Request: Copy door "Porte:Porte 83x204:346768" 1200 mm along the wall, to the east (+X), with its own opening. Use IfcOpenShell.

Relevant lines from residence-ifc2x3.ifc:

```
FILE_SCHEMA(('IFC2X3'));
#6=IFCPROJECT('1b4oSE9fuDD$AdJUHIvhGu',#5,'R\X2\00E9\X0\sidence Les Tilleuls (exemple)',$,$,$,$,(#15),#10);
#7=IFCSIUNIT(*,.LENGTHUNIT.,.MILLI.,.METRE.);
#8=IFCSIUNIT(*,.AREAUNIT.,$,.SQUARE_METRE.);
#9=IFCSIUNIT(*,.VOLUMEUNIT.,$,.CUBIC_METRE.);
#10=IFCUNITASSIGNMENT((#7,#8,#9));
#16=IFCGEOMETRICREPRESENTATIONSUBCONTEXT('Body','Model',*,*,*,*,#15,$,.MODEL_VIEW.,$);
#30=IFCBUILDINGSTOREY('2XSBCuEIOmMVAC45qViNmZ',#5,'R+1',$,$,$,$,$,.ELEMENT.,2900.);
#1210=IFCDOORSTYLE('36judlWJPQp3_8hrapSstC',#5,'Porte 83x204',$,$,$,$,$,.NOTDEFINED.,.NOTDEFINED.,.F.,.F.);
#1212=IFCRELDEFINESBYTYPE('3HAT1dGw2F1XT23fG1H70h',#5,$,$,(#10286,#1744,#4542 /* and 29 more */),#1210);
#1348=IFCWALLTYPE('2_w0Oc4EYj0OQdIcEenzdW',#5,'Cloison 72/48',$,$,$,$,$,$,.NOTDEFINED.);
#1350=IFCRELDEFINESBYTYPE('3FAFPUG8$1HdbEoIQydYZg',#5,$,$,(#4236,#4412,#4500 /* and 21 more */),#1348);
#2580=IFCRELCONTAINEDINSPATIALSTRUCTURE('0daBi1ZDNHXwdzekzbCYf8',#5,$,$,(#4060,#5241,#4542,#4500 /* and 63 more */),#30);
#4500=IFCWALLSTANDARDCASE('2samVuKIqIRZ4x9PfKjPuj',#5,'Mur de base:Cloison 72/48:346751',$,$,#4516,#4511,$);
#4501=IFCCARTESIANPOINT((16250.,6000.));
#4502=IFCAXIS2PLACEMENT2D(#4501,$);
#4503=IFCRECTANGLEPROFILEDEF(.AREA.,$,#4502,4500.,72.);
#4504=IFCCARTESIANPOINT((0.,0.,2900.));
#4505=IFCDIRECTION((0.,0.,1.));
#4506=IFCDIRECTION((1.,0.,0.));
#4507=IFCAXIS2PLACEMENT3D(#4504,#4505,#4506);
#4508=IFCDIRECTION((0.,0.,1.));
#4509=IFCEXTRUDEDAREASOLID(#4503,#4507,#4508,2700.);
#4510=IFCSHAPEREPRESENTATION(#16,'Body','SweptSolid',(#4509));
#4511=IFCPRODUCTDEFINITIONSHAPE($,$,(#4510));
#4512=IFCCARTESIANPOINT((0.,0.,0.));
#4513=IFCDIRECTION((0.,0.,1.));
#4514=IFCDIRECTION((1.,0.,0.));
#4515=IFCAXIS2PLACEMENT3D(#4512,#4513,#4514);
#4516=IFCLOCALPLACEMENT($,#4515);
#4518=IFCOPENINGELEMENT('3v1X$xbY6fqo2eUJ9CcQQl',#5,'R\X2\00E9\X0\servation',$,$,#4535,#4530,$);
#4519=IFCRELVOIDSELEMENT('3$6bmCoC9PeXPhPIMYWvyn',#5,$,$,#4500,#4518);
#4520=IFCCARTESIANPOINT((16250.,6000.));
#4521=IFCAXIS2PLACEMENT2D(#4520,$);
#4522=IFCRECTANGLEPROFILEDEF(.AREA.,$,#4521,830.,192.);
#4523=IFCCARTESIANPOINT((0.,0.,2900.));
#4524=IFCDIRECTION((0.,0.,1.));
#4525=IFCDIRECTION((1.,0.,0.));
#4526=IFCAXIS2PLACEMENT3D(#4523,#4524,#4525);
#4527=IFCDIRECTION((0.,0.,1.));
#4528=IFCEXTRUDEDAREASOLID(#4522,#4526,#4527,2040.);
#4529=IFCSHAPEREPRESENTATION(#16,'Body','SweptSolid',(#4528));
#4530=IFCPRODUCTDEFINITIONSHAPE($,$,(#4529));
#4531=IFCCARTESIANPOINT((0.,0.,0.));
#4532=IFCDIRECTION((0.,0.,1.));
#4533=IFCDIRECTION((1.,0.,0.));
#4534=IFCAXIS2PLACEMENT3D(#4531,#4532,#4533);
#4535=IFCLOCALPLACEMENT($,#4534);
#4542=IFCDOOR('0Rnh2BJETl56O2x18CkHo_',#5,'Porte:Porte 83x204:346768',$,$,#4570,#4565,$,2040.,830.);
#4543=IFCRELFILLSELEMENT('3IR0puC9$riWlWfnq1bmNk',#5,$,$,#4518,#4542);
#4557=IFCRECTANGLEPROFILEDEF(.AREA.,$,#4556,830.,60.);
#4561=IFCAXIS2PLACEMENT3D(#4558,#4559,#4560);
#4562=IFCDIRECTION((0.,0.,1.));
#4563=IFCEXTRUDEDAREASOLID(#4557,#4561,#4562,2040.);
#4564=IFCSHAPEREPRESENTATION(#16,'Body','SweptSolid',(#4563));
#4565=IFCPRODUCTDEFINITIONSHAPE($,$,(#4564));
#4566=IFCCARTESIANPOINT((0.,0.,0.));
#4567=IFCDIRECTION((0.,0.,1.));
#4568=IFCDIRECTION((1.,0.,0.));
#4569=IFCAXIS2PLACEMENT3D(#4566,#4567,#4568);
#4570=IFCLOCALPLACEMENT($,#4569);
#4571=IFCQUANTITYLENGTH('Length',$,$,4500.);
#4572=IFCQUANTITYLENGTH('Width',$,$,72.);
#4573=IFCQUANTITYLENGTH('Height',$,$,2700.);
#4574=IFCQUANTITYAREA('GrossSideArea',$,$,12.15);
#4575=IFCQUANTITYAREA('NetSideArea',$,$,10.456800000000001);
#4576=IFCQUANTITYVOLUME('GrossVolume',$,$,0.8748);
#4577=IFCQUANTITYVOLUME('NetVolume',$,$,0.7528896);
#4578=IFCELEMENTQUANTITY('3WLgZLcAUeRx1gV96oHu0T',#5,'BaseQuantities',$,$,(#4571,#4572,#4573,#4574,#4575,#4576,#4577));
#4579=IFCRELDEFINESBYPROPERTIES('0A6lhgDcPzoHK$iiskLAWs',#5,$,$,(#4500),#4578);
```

```python
import ifcopenshell
import ifcopenshell.api.feature
import ifcopenshell.api.geometry
import ifcopenshell.api.pset
import ifcopenshell.api.root
import ifcopenshell.geom
import ifcopenshell.util.element
import ifcopenshell.util.placement
import ifcopenshell.util.shape
import ifcopenshell.util.unit

model = ifcopenshell.open("residence-ifc2x3.ifc")
area_scale = ifcopenshell.util.unit.calculate_unit_scale(model, "AREAUNIT")
volume_scale = ifcopenshell.util.unit.calculate_unit_scale(model, "VOLUMEUNIT")
settings = ifcopenshell.geom.settings()


def volume(element):
    """Net volume in cubic metres, openings subtracted."""
    shape = ifcopenshell.geom.create_shape(settings, element)
    return ifcopenshell.util.shape.get_volume(shape.geometry)


def reuse_history(source, copy):
    """copy_class also copies each property set's owner history, people and application; keep the originals."""
    for rel in copy.IsDefinedBy:
        if rel.is_a("IfcRelDefinesByProperties") and (history := rel.RelatingPropertyDefinition.OwnerHistory):
            rel.RelatingPropertyDefinition.OwnerHistory = source.OwnerHistory
            ifcopenshell.util.element.remove_deep2(model, history)


door = model.by_guid("0Rnh2BJETl56O2x18CkHo_")
opening = door.FillsVoids[0].RelatingOpeningElement
wall = opening.VoidsElements[0].RelatingBuildingElement
before = volume(wall)
shift = ifcopenshell.util.placement.get_local_placement(wall.ObjectPlacement)[:3, 0] * 1200.0

# copy_class copies the void relationship, type, container and properties, but no geometry.
new_opening = ifcopenshell.api.root.copy_class(model, product=opening)
new_opening.Representation = ifcopenshell.util.element.copy_deep(
    model, opening.Representation, exclude=["IfcGeometricRepresentationContext", "IfcRepresentationMap"]
)
reuse_history(opening, new_opening)
new_door = ifcopenshell.api.root.copy_class(model, product=door)
new_door.Representation = ifcopenshell.util.element.copy_deep(
    model, door.Representation, exclude=["IfcGeometricRepresentationContext", "IfcRepresentationMap"]
)
new_door.Name = "Porte:Porte 83x204"
reuse_history(door, new_door)
fills = ifcopenshell.api.feature.add_filling(model, opening=new_opening, element=new_door)
fills.OwnerHistory = new_door.OwnerHistory  # required in IFC2X3

for old, new in ((opening, new_opening), (door, new_door)):
    matrix = ifcopenshell.util.placement.get_local_placement(old.ObjectPlacement)
    matrix[:3, 3] += shift
    ifcopenshell.api.geometry.edit_object_placement(model, product=new, matrix=matrix, is_si=False)

after = volume(wall)
thickness = 0.072  # wall thickness in metres

# Update the wall's stored quantities.
qto = model.by_id(ifcopenshell.util.element.get_pset(wall, "BaseQuantities", should_inherit=False)["id"])
ifcopenshell.api.pset.edit_qto(model, qto=qto, properties={
    "NetSideArea": after / thickness / area_scale,
    "NetVolume": after / volume_scale,
})

print(f"wall volume {before:.3f} -> {after:.3f} m3")

model.write("residence-ifc2x3_edited.ifc")
```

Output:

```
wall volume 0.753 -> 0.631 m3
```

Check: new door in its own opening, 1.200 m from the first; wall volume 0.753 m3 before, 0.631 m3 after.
